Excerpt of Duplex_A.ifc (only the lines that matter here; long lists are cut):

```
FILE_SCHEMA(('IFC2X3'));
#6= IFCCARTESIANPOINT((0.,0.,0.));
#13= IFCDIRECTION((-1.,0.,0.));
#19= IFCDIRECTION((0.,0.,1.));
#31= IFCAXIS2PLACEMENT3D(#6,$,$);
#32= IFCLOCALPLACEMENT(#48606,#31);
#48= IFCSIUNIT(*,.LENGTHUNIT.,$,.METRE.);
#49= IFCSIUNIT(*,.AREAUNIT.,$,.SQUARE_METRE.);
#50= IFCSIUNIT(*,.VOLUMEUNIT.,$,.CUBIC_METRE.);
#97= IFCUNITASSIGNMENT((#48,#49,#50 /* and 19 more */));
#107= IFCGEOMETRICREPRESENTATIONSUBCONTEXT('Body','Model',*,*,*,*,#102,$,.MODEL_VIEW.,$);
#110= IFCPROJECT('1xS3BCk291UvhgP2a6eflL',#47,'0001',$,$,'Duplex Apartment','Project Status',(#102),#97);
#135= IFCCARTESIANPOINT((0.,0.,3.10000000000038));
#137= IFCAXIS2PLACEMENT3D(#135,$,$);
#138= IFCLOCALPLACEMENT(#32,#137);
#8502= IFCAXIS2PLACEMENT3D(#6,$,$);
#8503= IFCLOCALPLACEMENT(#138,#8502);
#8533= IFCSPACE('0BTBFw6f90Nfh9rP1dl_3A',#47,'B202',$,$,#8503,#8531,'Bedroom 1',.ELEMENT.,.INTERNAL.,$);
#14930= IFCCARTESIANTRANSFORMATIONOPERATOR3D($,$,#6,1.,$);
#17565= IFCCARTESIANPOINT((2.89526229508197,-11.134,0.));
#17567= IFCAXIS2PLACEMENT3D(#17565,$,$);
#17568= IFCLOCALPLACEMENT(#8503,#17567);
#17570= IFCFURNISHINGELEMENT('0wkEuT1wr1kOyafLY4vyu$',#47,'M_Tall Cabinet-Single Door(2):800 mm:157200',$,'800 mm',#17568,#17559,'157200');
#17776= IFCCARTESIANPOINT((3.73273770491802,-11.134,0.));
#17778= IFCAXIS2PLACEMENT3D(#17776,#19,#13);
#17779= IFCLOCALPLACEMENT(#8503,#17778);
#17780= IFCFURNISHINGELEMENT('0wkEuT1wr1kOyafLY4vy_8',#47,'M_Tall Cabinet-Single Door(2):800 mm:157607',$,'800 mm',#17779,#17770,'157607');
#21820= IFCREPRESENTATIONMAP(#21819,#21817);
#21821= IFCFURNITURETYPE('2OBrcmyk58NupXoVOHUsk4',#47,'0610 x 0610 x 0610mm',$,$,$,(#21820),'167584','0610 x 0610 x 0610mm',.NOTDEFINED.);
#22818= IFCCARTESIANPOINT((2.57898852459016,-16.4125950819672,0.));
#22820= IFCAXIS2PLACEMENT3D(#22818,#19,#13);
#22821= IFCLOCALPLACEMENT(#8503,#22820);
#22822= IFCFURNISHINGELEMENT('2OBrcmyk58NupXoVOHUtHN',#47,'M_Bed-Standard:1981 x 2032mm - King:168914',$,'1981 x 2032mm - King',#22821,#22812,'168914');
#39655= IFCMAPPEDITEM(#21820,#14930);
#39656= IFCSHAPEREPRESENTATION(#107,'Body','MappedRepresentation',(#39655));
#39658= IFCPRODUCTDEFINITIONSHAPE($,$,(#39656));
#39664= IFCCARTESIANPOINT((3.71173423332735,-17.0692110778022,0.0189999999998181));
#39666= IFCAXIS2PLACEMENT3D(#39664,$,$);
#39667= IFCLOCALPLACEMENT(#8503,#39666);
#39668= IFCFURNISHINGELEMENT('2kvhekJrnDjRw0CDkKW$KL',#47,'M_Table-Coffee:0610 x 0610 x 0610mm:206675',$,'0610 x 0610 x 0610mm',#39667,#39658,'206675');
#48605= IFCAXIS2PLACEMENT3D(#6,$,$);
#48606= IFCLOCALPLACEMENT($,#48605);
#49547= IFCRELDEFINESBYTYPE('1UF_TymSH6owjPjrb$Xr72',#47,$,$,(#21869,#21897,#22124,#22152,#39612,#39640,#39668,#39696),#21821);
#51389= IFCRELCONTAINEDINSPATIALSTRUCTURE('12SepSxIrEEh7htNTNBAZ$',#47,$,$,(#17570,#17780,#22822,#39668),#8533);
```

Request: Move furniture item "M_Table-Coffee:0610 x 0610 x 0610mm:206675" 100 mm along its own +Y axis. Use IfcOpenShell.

```python
import ifcopenshell
import ifcopenshell.api.geometry
import ifcopenshell.util.placement

model = ifcopenshell.open("Duplex_A.ifc")

item = model.by_guid("2kvhekJrnDjRw0CDkKW$KL")
matrix = ifcopenshell.util.placement.get_local_placement(item.ObjectPlacement)
matrix[:3, 3] += matrix[:3, 1] * 0.1
ifcopenshell.api.geometry.edit_object_placement(model, product=item, matrix=matrix, is_si=False)

print(ifcopenshell.util.placement.get_local_placement(item.ObjectPlacement).round(3) + 0.0)

model.write("Duplex_A-out.ifc")
```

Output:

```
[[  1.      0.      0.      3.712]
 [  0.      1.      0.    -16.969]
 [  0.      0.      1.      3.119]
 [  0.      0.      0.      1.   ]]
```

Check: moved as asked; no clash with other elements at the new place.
